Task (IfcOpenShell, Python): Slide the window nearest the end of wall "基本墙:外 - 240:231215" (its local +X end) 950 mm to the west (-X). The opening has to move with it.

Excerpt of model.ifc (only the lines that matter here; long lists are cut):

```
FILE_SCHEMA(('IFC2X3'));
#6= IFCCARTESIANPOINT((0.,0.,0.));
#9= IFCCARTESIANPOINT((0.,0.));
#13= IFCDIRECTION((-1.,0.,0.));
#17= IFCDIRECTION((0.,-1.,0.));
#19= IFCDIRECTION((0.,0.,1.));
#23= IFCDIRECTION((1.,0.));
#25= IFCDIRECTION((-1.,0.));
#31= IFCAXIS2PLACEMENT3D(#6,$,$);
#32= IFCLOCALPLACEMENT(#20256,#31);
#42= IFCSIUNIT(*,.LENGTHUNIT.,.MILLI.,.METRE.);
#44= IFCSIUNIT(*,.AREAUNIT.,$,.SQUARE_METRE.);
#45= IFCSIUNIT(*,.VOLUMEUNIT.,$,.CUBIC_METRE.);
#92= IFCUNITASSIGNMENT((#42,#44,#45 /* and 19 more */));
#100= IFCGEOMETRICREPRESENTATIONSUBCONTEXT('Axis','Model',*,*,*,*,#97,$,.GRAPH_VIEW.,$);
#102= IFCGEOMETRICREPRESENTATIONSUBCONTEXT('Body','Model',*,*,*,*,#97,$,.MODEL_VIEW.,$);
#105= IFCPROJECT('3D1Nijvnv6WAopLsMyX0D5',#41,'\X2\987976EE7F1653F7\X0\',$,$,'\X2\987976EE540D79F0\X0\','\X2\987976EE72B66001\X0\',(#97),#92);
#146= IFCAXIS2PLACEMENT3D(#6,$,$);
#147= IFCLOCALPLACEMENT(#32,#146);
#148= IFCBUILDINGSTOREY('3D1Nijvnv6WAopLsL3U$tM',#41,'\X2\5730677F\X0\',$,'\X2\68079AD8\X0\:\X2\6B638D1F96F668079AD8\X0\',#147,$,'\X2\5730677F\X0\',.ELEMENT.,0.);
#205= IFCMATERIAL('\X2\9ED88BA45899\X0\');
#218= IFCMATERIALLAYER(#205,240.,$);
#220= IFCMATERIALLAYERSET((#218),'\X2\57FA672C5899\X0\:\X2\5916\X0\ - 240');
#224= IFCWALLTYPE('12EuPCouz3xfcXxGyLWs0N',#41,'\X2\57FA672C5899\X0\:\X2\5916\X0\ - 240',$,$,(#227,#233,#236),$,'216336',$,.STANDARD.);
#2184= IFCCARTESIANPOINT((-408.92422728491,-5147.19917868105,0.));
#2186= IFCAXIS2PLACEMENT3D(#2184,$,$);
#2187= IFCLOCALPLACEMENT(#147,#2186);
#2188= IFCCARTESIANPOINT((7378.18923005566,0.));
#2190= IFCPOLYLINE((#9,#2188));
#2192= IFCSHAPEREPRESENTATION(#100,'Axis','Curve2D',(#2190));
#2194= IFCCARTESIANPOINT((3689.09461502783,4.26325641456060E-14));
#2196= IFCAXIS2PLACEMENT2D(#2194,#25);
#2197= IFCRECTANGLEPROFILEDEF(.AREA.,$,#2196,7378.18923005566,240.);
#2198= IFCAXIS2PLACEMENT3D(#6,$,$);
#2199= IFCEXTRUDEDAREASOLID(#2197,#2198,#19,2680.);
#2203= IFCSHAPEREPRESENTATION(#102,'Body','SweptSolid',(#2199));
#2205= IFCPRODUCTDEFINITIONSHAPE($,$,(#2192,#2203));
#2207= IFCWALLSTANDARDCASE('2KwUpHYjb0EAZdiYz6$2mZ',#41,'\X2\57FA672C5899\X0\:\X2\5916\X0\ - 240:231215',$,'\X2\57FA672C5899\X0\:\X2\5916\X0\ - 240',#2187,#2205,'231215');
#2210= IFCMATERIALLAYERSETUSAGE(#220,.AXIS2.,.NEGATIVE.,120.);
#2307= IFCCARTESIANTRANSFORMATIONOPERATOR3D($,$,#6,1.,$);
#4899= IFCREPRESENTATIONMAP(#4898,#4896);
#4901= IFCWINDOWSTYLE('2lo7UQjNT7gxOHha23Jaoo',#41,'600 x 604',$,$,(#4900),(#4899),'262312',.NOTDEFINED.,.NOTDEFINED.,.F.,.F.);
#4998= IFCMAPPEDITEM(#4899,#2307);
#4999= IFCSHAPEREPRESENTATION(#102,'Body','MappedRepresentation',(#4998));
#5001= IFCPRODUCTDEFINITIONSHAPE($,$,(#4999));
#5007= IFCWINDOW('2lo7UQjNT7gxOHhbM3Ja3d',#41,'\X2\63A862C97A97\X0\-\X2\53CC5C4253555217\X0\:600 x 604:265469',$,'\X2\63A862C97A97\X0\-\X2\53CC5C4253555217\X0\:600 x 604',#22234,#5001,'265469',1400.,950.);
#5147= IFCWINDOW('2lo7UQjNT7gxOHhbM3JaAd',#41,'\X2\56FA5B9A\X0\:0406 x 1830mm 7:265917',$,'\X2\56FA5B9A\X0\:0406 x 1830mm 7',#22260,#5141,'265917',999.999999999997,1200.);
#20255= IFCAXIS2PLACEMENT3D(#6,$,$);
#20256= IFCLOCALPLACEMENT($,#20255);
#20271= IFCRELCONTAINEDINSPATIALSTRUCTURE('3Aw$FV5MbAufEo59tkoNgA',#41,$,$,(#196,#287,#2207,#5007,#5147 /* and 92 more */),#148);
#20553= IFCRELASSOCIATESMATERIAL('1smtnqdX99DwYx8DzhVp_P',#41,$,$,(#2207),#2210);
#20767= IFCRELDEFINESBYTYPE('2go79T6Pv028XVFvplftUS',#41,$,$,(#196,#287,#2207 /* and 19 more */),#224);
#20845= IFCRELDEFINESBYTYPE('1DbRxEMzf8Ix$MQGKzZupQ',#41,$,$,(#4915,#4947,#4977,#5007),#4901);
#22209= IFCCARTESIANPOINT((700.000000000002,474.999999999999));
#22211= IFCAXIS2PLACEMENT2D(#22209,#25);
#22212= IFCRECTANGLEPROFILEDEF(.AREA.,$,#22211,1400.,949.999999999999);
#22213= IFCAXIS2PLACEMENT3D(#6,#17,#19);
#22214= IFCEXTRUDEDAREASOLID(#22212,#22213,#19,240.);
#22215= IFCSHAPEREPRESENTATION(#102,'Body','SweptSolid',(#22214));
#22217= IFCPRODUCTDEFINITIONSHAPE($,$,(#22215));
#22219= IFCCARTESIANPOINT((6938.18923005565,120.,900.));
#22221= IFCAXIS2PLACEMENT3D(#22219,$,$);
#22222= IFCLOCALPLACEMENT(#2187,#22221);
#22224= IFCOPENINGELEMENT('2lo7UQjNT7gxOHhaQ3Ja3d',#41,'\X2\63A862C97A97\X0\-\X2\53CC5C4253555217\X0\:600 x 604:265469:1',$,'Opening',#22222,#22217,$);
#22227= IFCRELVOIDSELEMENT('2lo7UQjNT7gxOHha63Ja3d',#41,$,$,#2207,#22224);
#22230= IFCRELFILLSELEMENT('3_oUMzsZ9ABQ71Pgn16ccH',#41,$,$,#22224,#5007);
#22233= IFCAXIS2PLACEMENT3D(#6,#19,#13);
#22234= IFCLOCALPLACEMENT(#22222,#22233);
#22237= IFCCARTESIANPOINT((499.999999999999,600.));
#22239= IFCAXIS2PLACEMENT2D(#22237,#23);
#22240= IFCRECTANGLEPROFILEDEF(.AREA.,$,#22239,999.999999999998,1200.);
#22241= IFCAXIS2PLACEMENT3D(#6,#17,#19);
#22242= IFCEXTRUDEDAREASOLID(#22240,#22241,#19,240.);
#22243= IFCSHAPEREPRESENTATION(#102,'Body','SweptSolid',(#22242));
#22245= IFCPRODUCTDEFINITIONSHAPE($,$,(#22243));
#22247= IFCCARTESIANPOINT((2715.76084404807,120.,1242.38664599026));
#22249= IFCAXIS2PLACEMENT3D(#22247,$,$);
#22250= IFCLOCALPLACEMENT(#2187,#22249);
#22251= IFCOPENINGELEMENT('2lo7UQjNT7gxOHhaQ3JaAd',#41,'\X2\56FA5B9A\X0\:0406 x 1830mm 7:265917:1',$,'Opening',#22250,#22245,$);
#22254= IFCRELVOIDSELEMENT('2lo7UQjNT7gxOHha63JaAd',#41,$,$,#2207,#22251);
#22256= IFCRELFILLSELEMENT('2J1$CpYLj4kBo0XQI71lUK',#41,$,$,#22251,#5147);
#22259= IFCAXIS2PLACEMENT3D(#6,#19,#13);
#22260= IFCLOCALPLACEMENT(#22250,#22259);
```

```python
import ifcopenshell
import ifcopenshell.api.geometry
import ifcopenshell.util.placement
import ifcopenshell.util.unit

model = ifcopenshell.open("model.ifc")
unit_scale = ifcopenshell.util.unit.calculate_unit_scale(model)

window = model.by_id(5007)
opening = window.FillsVoids[0].RelatingOpeningElement
wall = opening.VoidsElements[0].RelatingBuildingElement

wall_matrix = ifcopenshell.util.placement.get_local_placement(wall.ObjectPlacement)
shift = wall_matrix[:3, 0] * -0.95 / unit_scale
before = ifcopenshell.util.placement.get_local_placement(window.ObjectPlacement)[:3, 3].copy()

# The window is placed relative to its opening, so it follows when the opening moves.
matrix = ifcopenshell.util.placement.get_local_placement(opening.ObjectPlacement)
matrix[:3, 3] += shift
ifcopenshell.api.geometry.edit_object_placement(
    model, product=opening, matrix=matrix, is_si=False, should_transform_children=True
)

after = ifcopenshell.util.placement.get_local_placement(window.ObjectPlacement)[:3, 3]
print("window moved by", (after - before).round(3) + 0.0)

model.write("model-out.ifc")
```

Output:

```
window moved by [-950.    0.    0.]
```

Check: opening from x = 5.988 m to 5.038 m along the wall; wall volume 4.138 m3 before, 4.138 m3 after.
